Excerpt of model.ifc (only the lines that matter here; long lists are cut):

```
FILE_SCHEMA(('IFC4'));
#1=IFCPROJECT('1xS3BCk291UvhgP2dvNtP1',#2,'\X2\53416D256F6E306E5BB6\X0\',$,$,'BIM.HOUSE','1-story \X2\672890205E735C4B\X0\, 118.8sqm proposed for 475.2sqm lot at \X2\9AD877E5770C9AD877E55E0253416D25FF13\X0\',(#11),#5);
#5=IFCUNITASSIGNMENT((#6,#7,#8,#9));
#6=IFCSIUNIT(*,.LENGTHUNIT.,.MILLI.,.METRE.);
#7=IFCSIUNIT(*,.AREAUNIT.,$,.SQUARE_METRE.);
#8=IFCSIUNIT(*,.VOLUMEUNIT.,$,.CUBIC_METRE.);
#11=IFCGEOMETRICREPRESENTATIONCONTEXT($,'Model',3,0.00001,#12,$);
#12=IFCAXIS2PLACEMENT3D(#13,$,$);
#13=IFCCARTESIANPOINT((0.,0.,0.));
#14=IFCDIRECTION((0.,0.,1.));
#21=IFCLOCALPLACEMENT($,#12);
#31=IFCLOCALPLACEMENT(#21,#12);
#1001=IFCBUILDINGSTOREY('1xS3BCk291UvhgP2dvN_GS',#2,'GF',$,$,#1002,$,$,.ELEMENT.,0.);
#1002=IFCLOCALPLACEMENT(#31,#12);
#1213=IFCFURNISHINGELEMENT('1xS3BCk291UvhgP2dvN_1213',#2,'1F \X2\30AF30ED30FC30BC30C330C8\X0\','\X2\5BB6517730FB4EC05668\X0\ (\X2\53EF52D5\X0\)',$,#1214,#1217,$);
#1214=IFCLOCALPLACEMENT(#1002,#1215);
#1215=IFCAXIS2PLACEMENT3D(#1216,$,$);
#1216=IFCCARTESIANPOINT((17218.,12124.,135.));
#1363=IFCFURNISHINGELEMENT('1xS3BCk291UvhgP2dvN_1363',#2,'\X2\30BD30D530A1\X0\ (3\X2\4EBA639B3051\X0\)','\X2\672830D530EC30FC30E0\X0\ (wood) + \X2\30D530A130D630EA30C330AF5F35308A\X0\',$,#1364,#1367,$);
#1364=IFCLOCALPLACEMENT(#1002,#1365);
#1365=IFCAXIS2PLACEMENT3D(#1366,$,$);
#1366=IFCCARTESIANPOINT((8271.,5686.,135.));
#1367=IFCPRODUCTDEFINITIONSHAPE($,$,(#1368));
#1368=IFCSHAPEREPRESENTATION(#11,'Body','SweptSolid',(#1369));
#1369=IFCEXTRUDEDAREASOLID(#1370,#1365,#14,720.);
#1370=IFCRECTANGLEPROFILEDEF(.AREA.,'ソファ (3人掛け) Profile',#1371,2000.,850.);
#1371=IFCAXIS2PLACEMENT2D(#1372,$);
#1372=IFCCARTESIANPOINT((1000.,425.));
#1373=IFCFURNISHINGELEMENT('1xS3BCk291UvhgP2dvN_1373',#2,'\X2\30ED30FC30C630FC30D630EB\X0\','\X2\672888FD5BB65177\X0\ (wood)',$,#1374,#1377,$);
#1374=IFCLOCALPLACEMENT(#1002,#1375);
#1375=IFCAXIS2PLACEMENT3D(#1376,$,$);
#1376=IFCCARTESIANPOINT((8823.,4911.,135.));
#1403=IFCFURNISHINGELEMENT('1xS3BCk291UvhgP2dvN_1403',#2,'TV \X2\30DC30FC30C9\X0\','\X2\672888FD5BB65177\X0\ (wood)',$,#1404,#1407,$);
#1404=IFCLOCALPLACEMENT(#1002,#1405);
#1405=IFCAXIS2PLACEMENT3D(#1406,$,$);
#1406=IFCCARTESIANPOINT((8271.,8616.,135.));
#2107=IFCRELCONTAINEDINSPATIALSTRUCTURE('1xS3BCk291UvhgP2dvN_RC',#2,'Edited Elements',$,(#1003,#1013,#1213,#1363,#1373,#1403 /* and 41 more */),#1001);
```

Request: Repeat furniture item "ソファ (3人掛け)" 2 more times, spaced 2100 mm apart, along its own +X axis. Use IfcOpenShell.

```python
import ifcopenshell
import ifcopenshell.api.geometry
import ifcopenshell.api.root
import ifcopenshell.util.element
import ifcopenshell.util.placement

model = ifcopenshell.open("model.ifc")


def reuse_history(source, copy):
    """copy_class also copies each property set's owner history, people and application; keep the originals."""
    for rel in copy.IsDefinedBy:
        if rel.is_a("IfcRelDefinesByProperties") and (history := rel.RelatingPropertyDefinition.OwnerHistory):
            rel.RelatingPropertyDefinition.OwnerHistory = source.OwnerHistory
            ifcopenshell.util.element.remove_deep2(model, history)


source = model.by_id(1363)
base = ifcopenshell.util.placement.get_local_placement(source.ObjectPlacement)
step = base[:3, 0] * 2100.0

for i in range(1, 3):
    copy = ifcopenshell.api.root.copy_class(model, product=source)
    copy.Representation = ifcopenshell.util.element.copy_deep(
        model, source.Representation, exclude=["IfcGeometricRepresentationContext", "IfcRepresentationMap"]
    )
    reuse_history(source, copy)
    matrix = base.copy()
    matrix[:3, 3] += i * step
    print("added at", matrix[:3, 3].round(3) + 0.0)
    ifcopenshell.api.geometry.edit_object_placement(model, product=copy, matrix=matrix, is_si=False)

model.write("model_updated.ifc")
```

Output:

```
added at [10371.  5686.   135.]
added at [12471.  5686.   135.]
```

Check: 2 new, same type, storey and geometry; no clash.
